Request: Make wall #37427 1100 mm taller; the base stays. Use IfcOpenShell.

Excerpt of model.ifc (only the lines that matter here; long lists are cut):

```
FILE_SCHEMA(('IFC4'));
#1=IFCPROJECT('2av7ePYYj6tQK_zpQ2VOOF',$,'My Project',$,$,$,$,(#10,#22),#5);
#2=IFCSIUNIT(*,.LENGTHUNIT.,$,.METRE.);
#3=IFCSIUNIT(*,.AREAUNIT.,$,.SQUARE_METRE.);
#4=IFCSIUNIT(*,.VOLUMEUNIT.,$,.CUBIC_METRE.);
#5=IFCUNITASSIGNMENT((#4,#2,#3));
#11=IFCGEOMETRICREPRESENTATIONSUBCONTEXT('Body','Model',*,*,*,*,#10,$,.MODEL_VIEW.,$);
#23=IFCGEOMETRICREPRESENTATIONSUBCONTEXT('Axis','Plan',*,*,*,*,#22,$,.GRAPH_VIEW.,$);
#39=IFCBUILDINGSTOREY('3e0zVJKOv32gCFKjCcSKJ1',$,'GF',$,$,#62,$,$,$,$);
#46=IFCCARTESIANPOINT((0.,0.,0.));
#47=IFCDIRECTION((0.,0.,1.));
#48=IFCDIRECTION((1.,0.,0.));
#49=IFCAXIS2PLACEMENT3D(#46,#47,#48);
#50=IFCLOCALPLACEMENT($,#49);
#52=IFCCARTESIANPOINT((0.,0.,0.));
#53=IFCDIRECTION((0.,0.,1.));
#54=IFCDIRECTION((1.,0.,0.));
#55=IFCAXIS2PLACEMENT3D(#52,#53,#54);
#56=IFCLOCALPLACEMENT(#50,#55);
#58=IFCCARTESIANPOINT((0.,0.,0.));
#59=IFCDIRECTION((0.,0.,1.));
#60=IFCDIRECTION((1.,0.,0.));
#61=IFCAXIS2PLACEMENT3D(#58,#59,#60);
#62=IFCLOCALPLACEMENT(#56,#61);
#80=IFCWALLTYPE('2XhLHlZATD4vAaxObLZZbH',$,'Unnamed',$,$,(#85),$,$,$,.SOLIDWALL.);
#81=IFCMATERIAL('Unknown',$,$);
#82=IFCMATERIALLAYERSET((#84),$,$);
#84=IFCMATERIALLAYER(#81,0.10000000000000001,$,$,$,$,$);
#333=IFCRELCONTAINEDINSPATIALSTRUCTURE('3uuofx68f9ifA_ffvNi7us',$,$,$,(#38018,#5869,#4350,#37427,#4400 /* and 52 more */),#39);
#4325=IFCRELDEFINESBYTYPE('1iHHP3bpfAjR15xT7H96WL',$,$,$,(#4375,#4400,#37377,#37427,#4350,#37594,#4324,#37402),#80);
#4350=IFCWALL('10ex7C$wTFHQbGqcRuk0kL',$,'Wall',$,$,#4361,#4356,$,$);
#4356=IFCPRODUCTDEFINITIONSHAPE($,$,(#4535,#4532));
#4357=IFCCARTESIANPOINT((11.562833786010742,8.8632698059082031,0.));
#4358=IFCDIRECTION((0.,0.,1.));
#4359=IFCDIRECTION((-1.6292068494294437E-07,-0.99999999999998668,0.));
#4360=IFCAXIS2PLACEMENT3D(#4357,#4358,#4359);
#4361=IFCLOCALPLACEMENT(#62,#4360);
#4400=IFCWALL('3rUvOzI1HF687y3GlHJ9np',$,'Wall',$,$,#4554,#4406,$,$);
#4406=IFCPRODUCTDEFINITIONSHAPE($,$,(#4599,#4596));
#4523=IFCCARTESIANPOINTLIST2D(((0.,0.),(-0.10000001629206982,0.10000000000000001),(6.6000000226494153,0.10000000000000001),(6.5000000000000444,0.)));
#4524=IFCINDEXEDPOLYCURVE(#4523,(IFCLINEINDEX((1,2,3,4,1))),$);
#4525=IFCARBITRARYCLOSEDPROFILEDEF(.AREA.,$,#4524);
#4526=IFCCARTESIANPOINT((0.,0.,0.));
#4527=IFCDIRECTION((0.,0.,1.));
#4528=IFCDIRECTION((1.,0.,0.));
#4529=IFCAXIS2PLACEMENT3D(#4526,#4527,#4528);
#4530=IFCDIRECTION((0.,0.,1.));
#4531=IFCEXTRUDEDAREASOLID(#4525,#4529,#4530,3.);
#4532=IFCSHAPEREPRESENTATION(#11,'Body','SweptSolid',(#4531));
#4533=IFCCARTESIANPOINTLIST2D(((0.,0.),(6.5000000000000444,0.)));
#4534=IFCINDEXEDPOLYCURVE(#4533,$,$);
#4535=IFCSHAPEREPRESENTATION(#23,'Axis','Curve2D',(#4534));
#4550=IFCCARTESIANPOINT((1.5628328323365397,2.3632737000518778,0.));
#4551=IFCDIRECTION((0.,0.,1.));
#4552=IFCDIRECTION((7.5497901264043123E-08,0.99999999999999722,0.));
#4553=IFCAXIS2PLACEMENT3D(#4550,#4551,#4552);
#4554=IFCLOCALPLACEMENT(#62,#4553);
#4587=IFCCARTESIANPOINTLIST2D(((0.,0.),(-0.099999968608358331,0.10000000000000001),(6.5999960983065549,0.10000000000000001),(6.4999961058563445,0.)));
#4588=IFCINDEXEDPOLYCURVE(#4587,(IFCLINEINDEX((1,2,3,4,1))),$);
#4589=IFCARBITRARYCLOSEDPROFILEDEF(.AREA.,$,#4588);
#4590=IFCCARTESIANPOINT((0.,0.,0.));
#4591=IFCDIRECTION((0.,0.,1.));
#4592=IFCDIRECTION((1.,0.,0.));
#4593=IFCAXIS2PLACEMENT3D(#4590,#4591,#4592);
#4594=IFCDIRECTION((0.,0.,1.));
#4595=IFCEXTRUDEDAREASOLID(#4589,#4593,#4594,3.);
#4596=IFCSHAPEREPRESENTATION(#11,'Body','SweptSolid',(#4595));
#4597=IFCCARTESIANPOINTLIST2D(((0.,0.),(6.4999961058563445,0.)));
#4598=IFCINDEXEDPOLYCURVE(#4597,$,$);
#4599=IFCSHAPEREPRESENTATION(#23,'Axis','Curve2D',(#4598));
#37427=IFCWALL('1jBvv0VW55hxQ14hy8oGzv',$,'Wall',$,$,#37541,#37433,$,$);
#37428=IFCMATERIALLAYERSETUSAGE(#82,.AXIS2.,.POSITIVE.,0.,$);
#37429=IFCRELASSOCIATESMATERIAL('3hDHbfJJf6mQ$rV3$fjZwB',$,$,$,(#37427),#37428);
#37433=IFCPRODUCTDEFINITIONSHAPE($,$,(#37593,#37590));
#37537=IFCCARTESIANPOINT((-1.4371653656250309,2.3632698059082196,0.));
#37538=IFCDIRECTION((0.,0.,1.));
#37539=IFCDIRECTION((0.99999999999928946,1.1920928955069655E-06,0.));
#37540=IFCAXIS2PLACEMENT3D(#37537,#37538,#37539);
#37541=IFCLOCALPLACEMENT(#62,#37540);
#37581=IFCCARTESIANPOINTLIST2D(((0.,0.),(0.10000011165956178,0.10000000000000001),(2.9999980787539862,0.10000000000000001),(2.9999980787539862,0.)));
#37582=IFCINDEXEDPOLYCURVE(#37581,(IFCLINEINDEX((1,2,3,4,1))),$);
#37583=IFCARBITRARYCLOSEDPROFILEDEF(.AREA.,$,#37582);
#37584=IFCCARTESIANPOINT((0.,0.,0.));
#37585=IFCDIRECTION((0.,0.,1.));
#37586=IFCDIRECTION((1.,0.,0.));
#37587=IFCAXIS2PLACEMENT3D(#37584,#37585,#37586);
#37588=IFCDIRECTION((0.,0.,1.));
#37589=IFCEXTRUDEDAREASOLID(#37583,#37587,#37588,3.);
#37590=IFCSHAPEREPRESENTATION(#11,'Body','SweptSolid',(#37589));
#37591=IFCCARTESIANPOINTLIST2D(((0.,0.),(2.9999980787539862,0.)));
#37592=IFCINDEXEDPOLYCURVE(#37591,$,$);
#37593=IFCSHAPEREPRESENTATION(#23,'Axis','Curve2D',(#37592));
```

```python
import ifcopenshell
import ifcopenshell.geom
import ifcopenshell.util.representation
import ifcopenshell.util.shape

model = ifcopenshell.open("model.ifc")
settings = ifcopenshell.geom.settings()


def volume(element):
    """Net volume in cubic metres, openings subtracted."""
    shape = ifcopenshell.geom.create_shape(settings, element)
    return ifcopenshell.util.shape.get_volume(shape.geometry)


wall = model.by_id(37427)
before = volume(wall)

body = ifcopenshell.util.representation.get_representation(wall, "Model", "Body")
solid = body.Items[0]
old_height = solid.Depth
solid.Depth += 1.1
after = volume(wall)

print(f"height {old_height:g} -> {solid.Depth:g}, volume {before:.3f} -> {after:.3f} m3")

model.write("model-out.ifc")
```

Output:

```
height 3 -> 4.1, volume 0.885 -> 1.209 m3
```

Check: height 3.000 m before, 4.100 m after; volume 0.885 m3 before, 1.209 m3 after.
